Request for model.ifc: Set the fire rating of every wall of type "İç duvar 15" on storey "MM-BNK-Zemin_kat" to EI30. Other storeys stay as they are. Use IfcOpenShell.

First a look at what the model holds.

```python
import ifcopenshell
import ifcopenshell.util.element

model = ifcopenshell.open("model.ifc")
print(model.schema)
storey = next(s for s in model.by_type("IfcBuildingStorey") if s.Name == "MM-BNK-Zemin_kat")
walls = [e for e in ifcopenshell.util.element.get_decomposition(storey) if e.is_a("IfcWall")]
seen = {}
for e in walls:
    element_type = ifcopenshell.util.element.get_type(e)
    key = (element_type.Name if element_type != e and element_type else None, ifcopenshell.util.element.get_pset(e, "Pset_WallCommon", "FireRating"))
    seen[key] = seen.get(key, 0) + 1
for (name, value), count in sorted(seen.items(), key=str):
    print(count, "x", name, "|", value)
```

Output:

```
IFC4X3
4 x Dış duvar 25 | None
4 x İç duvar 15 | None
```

```python
import ifcopenshell
import ifcopenshell.api.pset
import ifcopenshell.util.element

model = ifcopenshell.open("model.ifc")

storey = next(s for s in model.by_type("IfcBuildingStorey") if s.Name == "MM-BNK-Zemin_kat")
walls = [e for e in ifcopenshell.util.element.get_decomposition(storey) if e.is_a("IfcWall")]

count = 0
for e in walls:
    element_type = ifcopenshell.util.element.get_type(e)
    if element_type in (None, e) or element_type.Name != "İç duvar 15":
        continue
    # add_pset returns the element's existing set when there is one.
    pset = ifcopenshell.api.pset.add_pset(model, product=e, name="Pset_WallCommon")
    ifcopenshell.api.pset.edit_pset(model, pset=pset, properties={"FireRating": "EI30"})
    count += 1

print(count, "walls updated")

model.write("model-out.ifc")
```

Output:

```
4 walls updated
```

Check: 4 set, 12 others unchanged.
